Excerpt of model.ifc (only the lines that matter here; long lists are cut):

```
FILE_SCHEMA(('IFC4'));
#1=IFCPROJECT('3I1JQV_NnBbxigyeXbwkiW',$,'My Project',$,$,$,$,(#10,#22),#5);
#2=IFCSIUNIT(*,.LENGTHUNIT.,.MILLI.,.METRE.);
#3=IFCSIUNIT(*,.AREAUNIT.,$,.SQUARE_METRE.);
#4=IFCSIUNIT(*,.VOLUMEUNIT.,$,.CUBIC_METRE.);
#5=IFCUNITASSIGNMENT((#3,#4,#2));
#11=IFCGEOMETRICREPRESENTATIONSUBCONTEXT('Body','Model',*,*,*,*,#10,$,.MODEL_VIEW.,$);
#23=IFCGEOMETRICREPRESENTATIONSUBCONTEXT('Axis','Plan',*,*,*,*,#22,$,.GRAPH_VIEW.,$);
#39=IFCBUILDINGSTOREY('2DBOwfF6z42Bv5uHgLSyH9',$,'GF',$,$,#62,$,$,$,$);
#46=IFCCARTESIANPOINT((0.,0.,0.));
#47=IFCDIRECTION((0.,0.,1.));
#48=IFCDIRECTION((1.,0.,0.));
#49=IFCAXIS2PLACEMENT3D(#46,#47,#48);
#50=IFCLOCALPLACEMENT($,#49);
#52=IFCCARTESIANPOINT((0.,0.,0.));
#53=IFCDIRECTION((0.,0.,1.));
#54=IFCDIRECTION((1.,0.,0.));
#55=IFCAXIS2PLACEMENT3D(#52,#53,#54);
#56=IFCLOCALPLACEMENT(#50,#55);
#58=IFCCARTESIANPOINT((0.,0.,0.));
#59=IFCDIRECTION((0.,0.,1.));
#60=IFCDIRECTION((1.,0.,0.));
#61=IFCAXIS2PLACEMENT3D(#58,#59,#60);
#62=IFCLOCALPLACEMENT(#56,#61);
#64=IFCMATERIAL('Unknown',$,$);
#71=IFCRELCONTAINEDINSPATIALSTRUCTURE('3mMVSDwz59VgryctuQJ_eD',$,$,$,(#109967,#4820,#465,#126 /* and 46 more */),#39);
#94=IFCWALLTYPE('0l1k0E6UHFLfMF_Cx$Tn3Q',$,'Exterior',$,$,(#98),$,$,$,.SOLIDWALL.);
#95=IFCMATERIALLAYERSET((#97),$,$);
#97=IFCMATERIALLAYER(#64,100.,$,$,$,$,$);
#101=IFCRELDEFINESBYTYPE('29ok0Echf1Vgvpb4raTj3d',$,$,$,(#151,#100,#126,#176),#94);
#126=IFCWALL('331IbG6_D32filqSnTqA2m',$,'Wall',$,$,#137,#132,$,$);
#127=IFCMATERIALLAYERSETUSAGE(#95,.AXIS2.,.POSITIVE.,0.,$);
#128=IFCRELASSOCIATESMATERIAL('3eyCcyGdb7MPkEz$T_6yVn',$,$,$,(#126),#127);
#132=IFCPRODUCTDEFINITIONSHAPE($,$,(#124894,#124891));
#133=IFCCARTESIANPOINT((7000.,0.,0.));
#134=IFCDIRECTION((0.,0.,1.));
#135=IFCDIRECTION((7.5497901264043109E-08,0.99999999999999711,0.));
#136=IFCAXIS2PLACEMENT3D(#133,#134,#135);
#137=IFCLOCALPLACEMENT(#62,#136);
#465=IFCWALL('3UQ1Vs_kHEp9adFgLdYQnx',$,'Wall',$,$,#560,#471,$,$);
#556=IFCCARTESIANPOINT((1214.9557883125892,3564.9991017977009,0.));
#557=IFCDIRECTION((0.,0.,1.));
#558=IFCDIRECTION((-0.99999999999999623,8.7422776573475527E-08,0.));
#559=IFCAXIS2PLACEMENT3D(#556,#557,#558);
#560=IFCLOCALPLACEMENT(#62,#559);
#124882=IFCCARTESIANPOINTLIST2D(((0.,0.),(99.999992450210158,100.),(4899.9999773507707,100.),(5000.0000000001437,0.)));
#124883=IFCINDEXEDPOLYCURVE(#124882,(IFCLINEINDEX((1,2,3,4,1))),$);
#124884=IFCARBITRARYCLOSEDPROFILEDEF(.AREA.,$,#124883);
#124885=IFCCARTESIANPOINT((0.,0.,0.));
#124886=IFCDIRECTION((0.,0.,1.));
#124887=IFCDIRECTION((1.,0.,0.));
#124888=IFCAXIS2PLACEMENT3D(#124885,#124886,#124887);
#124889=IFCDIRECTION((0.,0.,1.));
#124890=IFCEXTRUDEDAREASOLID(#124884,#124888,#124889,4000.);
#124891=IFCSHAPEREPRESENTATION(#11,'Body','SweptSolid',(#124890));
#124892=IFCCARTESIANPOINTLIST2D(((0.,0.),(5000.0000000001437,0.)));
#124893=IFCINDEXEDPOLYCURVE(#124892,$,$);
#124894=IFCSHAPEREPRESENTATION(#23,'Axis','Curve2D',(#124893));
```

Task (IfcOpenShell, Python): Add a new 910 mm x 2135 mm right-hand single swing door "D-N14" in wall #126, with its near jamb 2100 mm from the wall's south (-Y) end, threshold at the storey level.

```python
import numpy as np
import ifcopenshell
import ifcopenshell.api.feature
import ifcopenshell.api.geometry
import ifcopenshell.api.root
import ifcopenshell.api.spatial
import ifcopenshell.geom
import ifcopenshell.util.element
import ifcopenshell.util.placement
import ifcopenshell.util.representation
import ifcopenshell.util.shape
import ifcopenshell.util.unit

model = ifcopenshell.open("model.ifc")
unit_scale = ifcopenshell.util.unit.calculate_unit_scale(model)
settings = ifcopenshell.geom.settings()


def volume(element):
    """Net volume in cubic metres, openings subtracted."""
    shape = ifcopenshell.geom.create_shape(settings, element)
    return ifcopenshell.util.shape.get_volume(shape.geometry)


wall = model.by_id(126)
storey = ifcopenshell.util.element.get_container(wall, ifc_class="IfcBuildingStorey")
context = ifcopenshell.util.representation.get_context(model, "Model", "Body", "MODEL_VIEW")
before = volume(wall)

width, height, from_end, sill = 0.91, 2.135, 2.1, 0.0  # metres

# The wall runs along its own X axis, and the end named is its -X end.
wall_shape = ifcopenshell.geom.create_shape(settings, wall)
x, y, z = ifcopenshell.util.shape.get_vertices(wall_shape.geometry).T
start = x.min() + from_end
face, thickness = float(y.min()), float(y.max() - y.min())
wall_matrix = ifcopenshell.util.placement.get_local_placement(wall.ObjectPlacement)
level = ifcopenshell.util.placement.get_local_placement(storey.ObjectPlacement)[2, 3]


def in_wall(x, y):
    """Placement at x, y metres in the wall's axes, at sill height."""
    matrix = wall_matrix.copy()
    matrix[:, 3] = wall_matrix @ np.array([x / unit_scale, y / unit_scale, 0.0, 1.0])
    matrix[2, 3] = level + sill / unit_scale
    return matrix


# Opening: a box that overshoots both wall faces by 50 mm.
opening = ifcopenshell.api.root.create_entity(model, ifc_class="IfcOpeningElement", predefined_type="OPENING")
box = ifcopenshell.api.geometry.add_wall_representation(
    model, context=context, length=width, height=height, thickness=thickness + 0.1
)
ifcopenshell.api.geometry.assign_representation(model, product=opening, representation=box)
ifcopenshell.api.geometry.edit_object_placement(model, product=opening, matrix=in_wall(start, face - 0.05), is_si=False)
ifcopenshell.api.feature.add_feature(model, feature=opening, element=wall)

door = ifcopenshell.api.root.create_entity(model, ifc_class="IfcDoor", name="D-N14", predefined_type="DOOR")
door.OverallWidth, door.OverallHeight = width / unit_scale, height / unit_scale
door.OperationType = "SINGLE_SWING_RIGHT"
body = ifcopenshell.api.geometry.add_door_representation(
    model,
    context=context,
    overall_width=door.OverallWidth,
    overall_height=door.OverallHeight,
    operation_type="SINGLE_SWING_RIGHT",
    lining_properties={"LiningDepth": thickness / unit_scale, "ThresholdDepth": thickness / unit_scale},
)
ifcopenshell.api.geometry.assign_representation(model, product=door, representation=body)
ifcopenshell.api.spatial.assign_container(model, products=[door], relating_structure=storey)
ifcopenshell.api.feature.add_filling(model, opening=opening, element=door)

# The lining spans the wall, so the door starts at the wall face.
ifcopenshell.api.geometry.edit_object_placement(model, product=door, matrix=in_wall(start, face), is_si=False)

after = volume(wall)

print(f"wall volume {before:.3f} -> {after:.3f} m3")

model.write("model_updated.ifc")
```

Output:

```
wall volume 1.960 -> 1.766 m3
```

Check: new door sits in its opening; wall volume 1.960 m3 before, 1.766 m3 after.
